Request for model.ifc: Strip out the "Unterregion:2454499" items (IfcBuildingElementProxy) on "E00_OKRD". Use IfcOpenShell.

First a look at what the model holds.

```python
import ifcopenshell
import ifcopenshell.util.element

model = ifcopenshell.open("model.ifc")
print(model.schema)
storey = next(s for s in model.by_type("IfcBuildingStorey") if s.Name == "E00_OKRD")
proxies = [e for e in ifcopenshell.util.element.get_decomposition(storey) if e.is_a("IfcBuildingElementProxy")]
seen = {}
for e in proxies:
    element_type = ifcopenshell.util.element.get_type(e)
    name = element_type.Name if element_type not in (None, e) else None
    seen[name] = seen.get(name, 0) + 1
for name, count in sorted(seen.items(), key=str):
    print(count, "x", name)
```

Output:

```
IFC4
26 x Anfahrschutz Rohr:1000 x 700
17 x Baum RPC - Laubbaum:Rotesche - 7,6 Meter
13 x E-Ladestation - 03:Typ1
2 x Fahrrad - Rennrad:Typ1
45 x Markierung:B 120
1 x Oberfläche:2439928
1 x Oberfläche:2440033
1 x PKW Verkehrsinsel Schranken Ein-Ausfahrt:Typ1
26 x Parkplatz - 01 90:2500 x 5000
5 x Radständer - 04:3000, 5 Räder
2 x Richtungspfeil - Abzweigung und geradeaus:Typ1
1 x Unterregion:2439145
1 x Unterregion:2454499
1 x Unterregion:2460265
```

```python
import ifcopenshell
import ifcopenshell.api.root
import ifcopenshell.util.element

model = ifcopenshell.open("model.ifc")

storey = next(s for s in model.by_type("IfcBuildingStorey") if s.Name == "E00_OKRD")
proxies = [e for e in ifcopenshell.util.element.get_decomposition(storey) if e.is_a("IfcBuildingElementProxy")]
targets = [e for e in proxies if (t := ifcopenshell.util.element.get_type(e)) not in (None, e) and t.Name == "Unterregion:2454499"]

for e in targets:
    ifcopenshell.api.root.remove_product(model, product=e)
print(len(targets), "removed")

model.write("model-out.ifc")
```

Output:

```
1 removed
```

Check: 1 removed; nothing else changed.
